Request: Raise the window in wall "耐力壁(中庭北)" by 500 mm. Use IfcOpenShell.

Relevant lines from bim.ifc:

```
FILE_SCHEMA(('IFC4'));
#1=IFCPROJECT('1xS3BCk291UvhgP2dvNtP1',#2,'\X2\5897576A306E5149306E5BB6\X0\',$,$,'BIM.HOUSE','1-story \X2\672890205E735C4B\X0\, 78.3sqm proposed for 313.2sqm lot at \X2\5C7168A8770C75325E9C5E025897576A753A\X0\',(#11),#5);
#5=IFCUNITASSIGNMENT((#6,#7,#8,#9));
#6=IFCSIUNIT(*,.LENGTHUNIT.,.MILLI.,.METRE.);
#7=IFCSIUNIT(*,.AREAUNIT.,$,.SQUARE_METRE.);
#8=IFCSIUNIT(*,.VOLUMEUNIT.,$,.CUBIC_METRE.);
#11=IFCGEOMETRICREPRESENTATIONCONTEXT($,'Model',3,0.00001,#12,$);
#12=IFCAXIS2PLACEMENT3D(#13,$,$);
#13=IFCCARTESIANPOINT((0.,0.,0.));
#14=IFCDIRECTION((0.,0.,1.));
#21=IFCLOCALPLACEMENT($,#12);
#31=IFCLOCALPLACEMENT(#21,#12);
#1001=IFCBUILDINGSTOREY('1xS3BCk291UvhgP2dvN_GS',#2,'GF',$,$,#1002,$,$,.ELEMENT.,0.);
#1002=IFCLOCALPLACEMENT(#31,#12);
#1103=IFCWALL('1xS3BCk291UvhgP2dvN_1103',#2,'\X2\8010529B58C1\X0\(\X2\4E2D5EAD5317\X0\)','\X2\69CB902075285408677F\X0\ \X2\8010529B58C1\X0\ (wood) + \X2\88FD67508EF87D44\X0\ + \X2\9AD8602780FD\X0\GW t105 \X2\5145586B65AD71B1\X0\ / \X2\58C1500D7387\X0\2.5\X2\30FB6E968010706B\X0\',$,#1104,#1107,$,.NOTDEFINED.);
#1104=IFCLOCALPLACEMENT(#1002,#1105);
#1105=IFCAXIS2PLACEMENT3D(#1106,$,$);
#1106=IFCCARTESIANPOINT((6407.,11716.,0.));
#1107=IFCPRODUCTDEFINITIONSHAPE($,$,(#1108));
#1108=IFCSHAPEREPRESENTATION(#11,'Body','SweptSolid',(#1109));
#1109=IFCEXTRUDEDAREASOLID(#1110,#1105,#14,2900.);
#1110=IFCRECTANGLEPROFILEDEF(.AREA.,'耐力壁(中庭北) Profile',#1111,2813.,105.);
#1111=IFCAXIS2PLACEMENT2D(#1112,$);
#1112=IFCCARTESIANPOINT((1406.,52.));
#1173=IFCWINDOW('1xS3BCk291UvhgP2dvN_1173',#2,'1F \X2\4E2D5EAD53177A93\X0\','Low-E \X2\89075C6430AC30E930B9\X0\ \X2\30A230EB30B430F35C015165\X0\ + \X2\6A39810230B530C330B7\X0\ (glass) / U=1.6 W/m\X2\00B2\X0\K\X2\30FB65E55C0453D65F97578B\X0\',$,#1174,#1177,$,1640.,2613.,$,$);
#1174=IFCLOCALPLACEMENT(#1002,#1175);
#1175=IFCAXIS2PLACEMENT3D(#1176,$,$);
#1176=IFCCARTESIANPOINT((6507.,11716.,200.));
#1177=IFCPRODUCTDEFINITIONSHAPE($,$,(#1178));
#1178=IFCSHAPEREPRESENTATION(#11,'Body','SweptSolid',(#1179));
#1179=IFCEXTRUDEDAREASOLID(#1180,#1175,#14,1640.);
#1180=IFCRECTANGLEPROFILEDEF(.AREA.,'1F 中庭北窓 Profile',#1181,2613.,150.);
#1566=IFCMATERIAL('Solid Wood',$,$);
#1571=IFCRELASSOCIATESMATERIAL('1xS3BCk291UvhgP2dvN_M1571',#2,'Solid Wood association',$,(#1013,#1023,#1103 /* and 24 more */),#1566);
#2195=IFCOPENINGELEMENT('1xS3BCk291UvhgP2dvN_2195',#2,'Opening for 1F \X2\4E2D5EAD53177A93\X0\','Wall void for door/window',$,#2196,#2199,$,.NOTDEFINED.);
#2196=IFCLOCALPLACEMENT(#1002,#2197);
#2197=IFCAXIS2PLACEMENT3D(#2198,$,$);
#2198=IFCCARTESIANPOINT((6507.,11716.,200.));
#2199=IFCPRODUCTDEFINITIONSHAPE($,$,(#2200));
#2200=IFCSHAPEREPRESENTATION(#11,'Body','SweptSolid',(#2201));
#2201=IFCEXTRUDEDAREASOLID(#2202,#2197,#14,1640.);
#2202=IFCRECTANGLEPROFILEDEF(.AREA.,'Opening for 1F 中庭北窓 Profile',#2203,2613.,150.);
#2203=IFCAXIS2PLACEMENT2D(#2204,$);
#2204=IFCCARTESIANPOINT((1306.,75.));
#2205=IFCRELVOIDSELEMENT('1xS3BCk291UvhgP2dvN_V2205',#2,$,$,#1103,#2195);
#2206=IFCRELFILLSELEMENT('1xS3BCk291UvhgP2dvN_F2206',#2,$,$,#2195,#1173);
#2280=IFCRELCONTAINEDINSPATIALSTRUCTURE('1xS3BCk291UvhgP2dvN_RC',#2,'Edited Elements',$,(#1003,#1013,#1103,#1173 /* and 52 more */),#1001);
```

```python
import numpy as np
import ifcopenshell
import ifcopenshell.api.geometry
import ifcopenshell.util.placement
import ifcopenshell.util.unit

model = ifcopenshell.open("bim.ifc")
unit_scale = ifcopenshell.util.unit.calculate_unit_scale(model)

window = model.by_guid("1xS3BCk291UvhgP2dvN_1173")
opening = window.FillsVoids[0].RelatingOpeningElement
dz = 0.5 / unit_scale

shift = np.array([0.0, 0.0, dz])
# The window is not placed relative to its opening, so move both.
for product in (opening, window):
    matrix = ifcopenshell.util.placement.get_local_placement(product.ObjectPlacement)
    matrix[:3, 3] += shift
    ifcopenshell.api.geometry.edit_object_placement(model, product=product, matrix=matrix, is_si=False)

print(f"moved by {dz * unit_scale:+.3f} m")

model.write("bim_edited.ifc")
```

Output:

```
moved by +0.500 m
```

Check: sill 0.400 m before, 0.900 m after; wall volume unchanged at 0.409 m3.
